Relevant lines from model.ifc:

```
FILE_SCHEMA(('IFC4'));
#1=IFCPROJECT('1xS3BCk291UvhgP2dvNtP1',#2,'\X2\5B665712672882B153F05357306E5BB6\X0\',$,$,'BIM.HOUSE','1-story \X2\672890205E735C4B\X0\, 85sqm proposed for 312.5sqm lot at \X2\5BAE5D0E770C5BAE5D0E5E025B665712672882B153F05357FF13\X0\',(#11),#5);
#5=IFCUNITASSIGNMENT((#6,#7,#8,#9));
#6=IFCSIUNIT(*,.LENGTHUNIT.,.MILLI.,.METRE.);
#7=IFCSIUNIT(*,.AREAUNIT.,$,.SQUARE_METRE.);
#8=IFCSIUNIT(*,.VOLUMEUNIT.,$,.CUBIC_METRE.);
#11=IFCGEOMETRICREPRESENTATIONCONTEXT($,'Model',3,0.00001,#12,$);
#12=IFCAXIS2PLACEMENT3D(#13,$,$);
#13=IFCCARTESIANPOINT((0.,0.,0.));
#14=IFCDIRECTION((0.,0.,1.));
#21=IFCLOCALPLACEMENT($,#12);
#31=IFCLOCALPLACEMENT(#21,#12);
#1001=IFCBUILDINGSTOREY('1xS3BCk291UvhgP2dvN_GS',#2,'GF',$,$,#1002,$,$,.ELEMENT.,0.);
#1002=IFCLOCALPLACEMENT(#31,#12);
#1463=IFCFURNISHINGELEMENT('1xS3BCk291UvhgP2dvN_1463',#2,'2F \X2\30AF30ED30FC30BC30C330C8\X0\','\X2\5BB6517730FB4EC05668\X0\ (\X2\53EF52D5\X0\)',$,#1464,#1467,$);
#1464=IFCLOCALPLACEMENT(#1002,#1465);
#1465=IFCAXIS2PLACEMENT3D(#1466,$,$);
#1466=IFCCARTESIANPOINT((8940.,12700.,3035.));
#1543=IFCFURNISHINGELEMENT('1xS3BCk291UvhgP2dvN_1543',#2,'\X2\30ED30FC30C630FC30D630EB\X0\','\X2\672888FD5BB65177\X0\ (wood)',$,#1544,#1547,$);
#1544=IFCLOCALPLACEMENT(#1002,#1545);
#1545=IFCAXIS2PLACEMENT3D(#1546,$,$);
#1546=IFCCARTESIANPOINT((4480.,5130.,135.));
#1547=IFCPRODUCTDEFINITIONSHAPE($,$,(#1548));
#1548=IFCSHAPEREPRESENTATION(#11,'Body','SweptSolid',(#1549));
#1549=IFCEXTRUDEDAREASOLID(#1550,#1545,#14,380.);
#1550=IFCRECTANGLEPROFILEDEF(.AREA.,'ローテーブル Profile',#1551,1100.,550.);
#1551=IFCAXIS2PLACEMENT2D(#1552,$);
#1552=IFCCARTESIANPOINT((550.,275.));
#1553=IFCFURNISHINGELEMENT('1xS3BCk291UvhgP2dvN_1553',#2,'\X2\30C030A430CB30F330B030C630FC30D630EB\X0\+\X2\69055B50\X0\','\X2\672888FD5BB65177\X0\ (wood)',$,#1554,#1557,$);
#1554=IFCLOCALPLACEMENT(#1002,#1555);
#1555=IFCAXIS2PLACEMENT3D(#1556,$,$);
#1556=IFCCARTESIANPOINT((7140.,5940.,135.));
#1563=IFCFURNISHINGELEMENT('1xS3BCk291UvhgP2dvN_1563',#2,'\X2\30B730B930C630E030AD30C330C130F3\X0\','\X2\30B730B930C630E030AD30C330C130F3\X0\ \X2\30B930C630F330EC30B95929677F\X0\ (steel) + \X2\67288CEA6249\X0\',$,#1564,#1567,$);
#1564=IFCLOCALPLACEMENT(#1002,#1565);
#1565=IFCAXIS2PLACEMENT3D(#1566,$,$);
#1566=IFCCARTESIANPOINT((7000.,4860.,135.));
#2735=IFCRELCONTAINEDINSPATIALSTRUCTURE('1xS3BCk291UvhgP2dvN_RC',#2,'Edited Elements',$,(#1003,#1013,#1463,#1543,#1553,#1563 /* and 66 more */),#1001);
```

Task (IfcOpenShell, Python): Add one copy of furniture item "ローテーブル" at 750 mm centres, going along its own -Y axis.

```python
import ifcopenshell
import ifcopenshell.api.geometry
import ifcopenshell.api.root
import ifcopenshell.util.element
import ifcopenshell.util.placement
import ifcopenshell.util.unit

model = ifcopenshell.open("model.ifc")
unit_scale = ifcopenshell.util.unit.calculate_unit_scale(model)


def reuse_history(source, copy):
    """copy_class also copies each property set's owner history, people and application; keep the originals."""
    for rel in copy.IsDefinedBy:
        if rel.is_a("IfcRelDefinesByProperties") and (history := rel.RelatingPropertyDefinition.OwnerHistory):
            rel.RelatingPropertyDefinition.OwnerHistory = source.OwnerHistory
            ifcopenshell.util.element.remove_deep2(model, history)


source = model.by_guid("1xS3BCk291UvhgP2dvN_1543")
base = ifcopenshell.util.placement.get_local_placement(source.ObjectPlacement)
step = -base[:3, 1] * 0.75 / unit_scale

for i in range(1, 2):
    copy = ifcopenshell.api.root.copy_class(model, product=source)
    copy.Representation = ifcopenshell.util.element.copy_deep(
        model, source.Representation, exclude=["IfcGeometricRepresentationContext", "IfcRepresentationMap"]
    )
    reuse_history(source, copy)
    matrix = base.copy()
    matrix[:3, 3] += i * step
    print("added at", matrix[:3, 3].round(3) + 0.0)
    ifcopenshell.api.geometry.edit_object_placement(model, product=copy, matrix=matrix, is_si=False)

model.write("model_edited.ifc")
```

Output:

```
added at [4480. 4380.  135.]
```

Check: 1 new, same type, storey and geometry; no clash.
